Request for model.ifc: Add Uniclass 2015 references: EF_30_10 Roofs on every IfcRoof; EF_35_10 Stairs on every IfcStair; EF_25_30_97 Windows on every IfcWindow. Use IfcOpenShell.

First a look at what the model holds.

```python
import ifcopenshell

model = ifcopenshell.open("model.ifc")
print(model.schema)
print("classifications:", [c.Name for c in model.by_type("IfcClassification")])
for ifc_class in ("IfcDoor", "IfcRoof", "IfcStair", "IfcWall", "IfcWindow"):
    print(ifc_class, len(model.by_type(ifc_class)))
```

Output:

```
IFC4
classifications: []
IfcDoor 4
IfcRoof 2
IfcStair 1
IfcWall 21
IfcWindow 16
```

```python
import ifcopenshell
import ifcopenshell.api.classification

model = ifcopenshell.open("model.ifc")

system = ifcopenshell.api.classification.add_classification(model, classification="Uniclass 2015")

codes = {
    "IfcRoof": ("EF_30_10", "Roofs"),
    "IfcStair": ("EF_35_10", "Stairs"),
    "IfcWindow": ("EF_25_30_97", "Windows"),
}
for ifc_class, (code, name) in codes.items():
    products = model.by_type(ifc_class)
    ifcopenshell.api.classification.add_reference(
        model, products=products, classification=system, identification=code, name=name
    )
    print(code, len(products))

model.write("model_edited.ifc")
```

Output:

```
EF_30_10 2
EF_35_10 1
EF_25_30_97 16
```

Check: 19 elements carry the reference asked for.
